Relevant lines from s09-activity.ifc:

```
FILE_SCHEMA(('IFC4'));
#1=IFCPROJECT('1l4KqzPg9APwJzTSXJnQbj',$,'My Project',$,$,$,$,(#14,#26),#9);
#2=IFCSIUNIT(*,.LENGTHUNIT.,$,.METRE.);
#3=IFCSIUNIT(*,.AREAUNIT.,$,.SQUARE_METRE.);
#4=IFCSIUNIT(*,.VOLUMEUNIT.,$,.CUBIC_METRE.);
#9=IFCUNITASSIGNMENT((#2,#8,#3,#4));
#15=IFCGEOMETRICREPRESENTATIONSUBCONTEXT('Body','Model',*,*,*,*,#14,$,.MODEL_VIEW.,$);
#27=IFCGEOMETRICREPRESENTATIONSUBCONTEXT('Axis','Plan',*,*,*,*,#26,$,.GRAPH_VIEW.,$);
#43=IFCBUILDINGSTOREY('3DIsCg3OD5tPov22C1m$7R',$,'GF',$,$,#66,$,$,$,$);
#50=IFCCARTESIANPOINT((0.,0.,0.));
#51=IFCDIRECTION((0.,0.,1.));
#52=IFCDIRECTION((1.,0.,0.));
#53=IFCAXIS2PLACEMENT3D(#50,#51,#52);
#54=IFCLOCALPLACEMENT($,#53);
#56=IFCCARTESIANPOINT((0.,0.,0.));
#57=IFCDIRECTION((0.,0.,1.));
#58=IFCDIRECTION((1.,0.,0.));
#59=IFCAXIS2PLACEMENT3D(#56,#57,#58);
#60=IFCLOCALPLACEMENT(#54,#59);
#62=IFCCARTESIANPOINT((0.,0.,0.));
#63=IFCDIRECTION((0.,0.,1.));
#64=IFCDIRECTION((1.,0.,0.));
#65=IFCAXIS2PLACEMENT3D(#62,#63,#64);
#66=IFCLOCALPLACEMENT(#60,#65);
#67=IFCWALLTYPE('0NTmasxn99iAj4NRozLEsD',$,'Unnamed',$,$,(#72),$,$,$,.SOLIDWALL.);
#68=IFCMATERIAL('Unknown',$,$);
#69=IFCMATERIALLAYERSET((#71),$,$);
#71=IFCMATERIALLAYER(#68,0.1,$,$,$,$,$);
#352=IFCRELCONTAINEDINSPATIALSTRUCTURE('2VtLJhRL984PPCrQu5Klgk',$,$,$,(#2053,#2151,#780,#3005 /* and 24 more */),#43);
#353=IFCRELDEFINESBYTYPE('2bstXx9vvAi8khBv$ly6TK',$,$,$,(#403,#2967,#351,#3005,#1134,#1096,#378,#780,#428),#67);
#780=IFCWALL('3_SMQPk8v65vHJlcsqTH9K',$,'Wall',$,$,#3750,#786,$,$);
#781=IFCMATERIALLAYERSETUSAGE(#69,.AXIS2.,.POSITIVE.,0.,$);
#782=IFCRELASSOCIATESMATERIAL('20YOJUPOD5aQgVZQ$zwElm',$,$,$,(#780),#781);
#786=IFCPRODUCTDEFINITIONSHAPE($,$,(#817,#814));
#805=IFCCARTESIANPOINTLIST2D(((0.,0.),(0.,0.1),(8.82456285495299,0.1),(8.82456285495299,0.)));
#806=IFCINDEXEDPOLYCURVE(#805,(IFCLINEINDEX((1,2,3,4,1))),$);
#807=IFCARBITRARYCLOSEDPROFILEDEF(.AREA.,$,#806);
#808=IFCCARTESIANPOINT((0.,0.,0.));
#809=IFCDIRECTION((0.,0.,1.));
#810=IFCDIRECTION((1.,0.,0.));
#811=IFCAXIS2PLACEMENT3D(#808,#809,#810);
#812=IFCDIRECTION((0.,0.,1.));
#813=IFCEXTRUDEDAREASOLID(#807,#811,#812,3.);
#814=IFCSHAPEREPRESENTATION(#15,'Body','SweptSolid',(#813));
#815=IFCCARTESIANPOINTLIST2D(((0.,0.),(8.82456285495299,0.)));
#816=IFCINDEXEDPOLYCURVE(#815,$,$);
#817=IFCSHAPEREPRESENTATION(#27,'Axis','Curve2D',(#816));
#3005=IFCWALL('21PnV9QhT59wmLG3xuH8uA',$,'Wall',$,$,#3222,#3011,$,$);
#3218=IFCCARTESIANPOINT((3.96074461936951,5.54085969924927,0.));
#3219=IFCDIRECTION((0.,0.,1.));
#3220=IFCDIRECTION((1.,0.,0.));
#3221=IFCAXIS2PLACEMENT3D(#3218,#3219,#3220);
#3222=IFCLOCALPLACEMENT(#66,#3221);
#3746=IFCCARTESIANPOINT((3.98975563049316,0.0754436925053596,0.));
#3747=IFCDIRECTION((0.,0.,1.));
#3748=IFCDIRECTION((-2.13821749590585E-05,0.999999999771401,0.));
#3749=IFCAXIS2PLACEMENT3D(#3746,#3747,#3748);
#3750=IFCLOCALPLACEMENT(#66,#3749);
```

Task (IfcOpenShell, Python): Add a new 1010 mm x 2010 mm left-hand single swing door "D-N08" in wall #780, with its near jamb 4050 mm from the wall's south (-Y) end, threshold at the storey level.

```python
import numpy as np
import ifcopenshell
import ifcopenshell.api.feature
import ifcopenshell.api.geometry
import ifcopenshell.api.root
import ifcopenshell.api.spatial
import ifcopenshell.geom
import ifcopenshell.util.element
import ifcopenshell.util.placement
import ifcopenshell.util.representation
import ifcopenshell.util.shape
import ifcopenshell.util.unit

model = ifcopenshell.open("s09-activity.ifc")
unit_scale = ifcopenshell.util.unit.calculate_unit_scale(model)
settings = ifcopenshell.geom.settings()


def volume(element):
    """Net volume in cubic metres, openings subtracted."""
    shape = ifcopenshell.geom.create_shape(settings, element)
    return ifcopenshell.util.shape.get_volume(shape.geometry)


wall = model.by_guid("3_SMQPk8v65vHJlcsqTH9K")
storey = ifcopenshell.util.element.get_container(wall, ifc_class="IfcBuildingStorey")
context = ifcopenshell.util.representation.get_context(model, "Model", "Body", "MODEL_VIEW")
before = volume(wall)

width, height, from_end, sill = 1.01, 2.01, 4.05, 0.0  # metres

# The wall runs along its own X axis, and the end named is its -X end.
wall_shape = ifcopenshell.geom.create_shape(settings, wall)
x, y, z = ifcopenshell.util.shape.get_vertices(wall_shape.geometry).T
start = x.min() + from_end
face, thickness = float(y.min()), float(y.max() - y.min())
wall_matrix = ifcopenshell.util.placement.get_local_placement(wall.ObjectPlacement)
level = ifcopenshell.util.placement.get_local_placement(storey.ObjectPlacement)[2, 3]


def in_wall(x, y):
    """Placement at x, y metres in the wall's axes, at sill height."""
    matrix = wall_matrix.copy()
    matrix[:, 3] = wall_matrix @ np.array([x / unit_scale, y / unit_scale, 0.0, 1.0])
    matrix[2, 3] = level + sill / unit_scale
    return matrix


# Opening: a box that overshoots both wall faces by 50 mm.
opening = ifcopenshell.api.root.create_entity(model, ifc_class="IfcOpeningElement", predefined_type="OPENING")
box = ifcopenshell.api.geometry.add_wall_representation(
    model, context=context, length=width, height=height, thickness=thickness + 0.1
)
ifcopenshell.api.geometry.assign_representation(model, product=opening, representation=box)
ifcopenshell.api.geometry.edit_object_placement(model, product=opening, matrix=in_wall(start, face - 0.05), is_si=False)
ifcopenshell.api.feature.add_feature(model, feature=opening, element=wall)

door = ifcopenshell.api.root.create_entity(model, ifc_class="IfcDoor", name="D-N08", predefined_type="DOOR")
door.OverallWidth, door.OverallHeight = width / unit_scale, height / unit_scale
door.OperationType = "SINGLE_SWING_LEFT"
body = ifcopenshell.api.geometry.add_door_representation(
    model,
    context=context,
    overall_width=door.OverallWidth,
    overall_height=door.OverallHeight,
    operation_type="SINGLE_SWING_LEFT",
    lining_properties={"LiningDepth": thickness / unit_scale, "ThresholdDepth": thickness / unit_scale},
)
ifcopenshell.api.geometry.assign_representation(model, product=door, representation=body)
ifcopenshell.api.spatial.assign_container(model, products=[door], relating_structure=storey)
ifcopenshell.api.feature.add_filling(model, opening=opening, element=door)

# The lining spans the wall, so the door starts at the wall face.
ifcopenshell.api.geometry.edit_object_placement(model, product=door, matrix=in_wall(start, face), is_si=False)

after = volume(wall)

print(f"wall volume {before:.3f} -> {after:.3f} m3")

model.write("s09-activity_edited.ifc")
```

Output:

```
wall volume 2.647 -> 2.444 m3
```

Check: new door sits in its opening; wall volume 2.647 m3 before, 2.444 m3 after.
